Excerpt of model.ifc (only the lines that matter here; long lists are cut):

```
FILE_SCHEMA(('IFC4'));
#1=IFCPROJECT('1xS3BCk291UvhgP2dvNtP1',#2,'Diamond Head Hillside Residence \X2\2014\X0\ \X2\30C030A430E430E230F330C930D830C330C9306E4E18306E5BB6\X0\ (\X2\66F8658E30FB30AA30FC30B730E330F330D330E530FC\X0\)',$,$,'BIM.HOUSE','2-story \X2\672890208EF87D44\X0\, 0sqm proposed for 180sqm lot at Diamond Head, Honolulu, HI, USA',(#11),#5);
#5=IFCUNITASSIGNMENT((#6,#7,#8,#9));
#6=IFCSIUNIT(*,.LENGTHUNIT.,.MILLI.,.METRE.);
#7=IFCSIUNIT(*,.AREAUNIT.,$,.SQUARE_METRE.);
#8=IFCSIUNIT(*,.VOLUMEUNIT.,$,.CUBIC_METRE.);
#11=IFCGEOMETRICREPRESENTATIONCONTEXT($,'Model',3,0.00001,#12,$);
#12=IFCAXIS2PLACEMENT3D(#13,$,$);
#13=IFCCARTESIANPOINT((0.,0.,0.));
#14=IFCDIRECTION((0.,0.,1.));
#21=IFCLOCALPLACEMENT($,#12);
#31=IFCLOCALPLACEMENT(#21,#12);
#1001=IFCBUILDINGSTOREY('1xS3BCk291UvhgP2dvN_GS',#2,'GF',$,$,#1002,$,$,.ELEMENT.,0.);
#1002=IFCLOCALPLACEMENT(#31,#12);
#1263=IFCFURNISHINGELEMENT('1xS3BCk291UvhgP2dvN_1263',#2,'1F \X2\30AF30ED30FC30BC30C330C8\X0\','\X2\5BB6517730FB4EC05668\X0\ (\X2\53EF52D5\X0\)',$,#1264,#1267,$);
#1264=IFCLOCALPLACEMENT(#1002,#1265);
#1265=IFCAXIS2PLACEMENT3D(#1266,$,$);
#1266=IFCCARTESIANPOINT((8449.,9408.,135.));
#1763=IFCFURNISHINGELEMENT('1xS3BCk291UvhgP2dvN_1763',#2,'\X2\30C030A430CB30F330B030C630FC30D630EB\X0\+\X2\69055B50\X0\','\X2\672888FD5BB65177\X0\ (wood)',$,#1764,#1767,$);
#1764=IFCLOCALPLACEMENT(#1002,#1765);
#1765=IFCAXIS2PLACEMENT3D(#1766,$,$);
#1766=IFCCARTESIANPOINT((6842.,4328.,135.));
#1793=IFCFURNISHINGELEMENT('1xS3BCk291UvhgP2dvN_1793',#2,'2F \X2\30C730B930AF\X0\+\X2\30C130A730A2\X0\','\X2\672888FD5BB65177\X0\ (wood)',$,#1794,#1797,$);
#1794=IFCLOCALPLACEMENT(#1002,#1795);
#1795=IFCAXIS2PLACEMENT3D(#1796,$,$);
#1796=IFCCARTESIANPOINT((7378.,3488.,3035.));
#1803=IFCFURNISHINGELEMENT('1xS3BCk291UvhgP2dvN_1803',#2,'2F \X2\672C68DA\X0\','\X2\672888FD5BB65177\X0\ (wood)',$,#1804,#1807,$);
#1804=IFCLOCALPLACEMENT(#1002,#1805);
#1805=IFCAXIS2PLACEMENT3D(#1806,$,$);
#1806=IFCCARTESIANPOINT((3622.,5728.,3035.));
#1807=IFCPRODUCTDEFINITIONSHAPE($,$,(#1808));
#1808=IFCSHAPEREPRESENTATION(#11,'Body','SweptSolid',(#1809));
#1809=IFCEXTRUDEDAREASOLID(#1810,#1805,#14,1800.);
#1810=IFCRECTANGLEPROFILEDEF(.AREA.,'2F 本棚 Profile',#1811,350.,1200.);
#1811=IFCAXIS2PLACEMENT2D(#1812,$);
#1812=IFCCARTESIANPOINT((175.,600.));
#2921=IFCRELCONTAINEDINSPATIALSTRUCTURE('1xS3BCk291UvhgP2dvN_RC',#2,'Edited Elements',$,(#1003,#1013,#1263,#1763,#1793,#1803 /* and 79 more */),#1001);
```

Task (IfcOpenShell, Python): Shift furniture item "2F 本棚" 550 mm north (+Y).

```python
import ifcopenshell
import ifcopenshell.api.geometry
import ifcopenshell.util.placement
import ifcopenshell.util.unit

model = ifcopenshell.open("model.ifc")
unit_scale = ifcopenshell.util.unit.calculate_unit_scale(model)

item = model.by_guid("1xS3BCk291UvhgP2dvN_1803")
matrix = ifcopenshell.util.placement.get_local_placement(item.ObjectPlacement)
matrix[1, 3] += 0.55 / unit_scale
ifcopenshell.api.geometry.edit_object_placement(model, product=item, matrix=matrix, is_si=False)

print(ifcopenshell.util.placement.get_local_placement(item.ObjectPlacement).round(3) + 0.0)

model.write("model-out.ifc")
```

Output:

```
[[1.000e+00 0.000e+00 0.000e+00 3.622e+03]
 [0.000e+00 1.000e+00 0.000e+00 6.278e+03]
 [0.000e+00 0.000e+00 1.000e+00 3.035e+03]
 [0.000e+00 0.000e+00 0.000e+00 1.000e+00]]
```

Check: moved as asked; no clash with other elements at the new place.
